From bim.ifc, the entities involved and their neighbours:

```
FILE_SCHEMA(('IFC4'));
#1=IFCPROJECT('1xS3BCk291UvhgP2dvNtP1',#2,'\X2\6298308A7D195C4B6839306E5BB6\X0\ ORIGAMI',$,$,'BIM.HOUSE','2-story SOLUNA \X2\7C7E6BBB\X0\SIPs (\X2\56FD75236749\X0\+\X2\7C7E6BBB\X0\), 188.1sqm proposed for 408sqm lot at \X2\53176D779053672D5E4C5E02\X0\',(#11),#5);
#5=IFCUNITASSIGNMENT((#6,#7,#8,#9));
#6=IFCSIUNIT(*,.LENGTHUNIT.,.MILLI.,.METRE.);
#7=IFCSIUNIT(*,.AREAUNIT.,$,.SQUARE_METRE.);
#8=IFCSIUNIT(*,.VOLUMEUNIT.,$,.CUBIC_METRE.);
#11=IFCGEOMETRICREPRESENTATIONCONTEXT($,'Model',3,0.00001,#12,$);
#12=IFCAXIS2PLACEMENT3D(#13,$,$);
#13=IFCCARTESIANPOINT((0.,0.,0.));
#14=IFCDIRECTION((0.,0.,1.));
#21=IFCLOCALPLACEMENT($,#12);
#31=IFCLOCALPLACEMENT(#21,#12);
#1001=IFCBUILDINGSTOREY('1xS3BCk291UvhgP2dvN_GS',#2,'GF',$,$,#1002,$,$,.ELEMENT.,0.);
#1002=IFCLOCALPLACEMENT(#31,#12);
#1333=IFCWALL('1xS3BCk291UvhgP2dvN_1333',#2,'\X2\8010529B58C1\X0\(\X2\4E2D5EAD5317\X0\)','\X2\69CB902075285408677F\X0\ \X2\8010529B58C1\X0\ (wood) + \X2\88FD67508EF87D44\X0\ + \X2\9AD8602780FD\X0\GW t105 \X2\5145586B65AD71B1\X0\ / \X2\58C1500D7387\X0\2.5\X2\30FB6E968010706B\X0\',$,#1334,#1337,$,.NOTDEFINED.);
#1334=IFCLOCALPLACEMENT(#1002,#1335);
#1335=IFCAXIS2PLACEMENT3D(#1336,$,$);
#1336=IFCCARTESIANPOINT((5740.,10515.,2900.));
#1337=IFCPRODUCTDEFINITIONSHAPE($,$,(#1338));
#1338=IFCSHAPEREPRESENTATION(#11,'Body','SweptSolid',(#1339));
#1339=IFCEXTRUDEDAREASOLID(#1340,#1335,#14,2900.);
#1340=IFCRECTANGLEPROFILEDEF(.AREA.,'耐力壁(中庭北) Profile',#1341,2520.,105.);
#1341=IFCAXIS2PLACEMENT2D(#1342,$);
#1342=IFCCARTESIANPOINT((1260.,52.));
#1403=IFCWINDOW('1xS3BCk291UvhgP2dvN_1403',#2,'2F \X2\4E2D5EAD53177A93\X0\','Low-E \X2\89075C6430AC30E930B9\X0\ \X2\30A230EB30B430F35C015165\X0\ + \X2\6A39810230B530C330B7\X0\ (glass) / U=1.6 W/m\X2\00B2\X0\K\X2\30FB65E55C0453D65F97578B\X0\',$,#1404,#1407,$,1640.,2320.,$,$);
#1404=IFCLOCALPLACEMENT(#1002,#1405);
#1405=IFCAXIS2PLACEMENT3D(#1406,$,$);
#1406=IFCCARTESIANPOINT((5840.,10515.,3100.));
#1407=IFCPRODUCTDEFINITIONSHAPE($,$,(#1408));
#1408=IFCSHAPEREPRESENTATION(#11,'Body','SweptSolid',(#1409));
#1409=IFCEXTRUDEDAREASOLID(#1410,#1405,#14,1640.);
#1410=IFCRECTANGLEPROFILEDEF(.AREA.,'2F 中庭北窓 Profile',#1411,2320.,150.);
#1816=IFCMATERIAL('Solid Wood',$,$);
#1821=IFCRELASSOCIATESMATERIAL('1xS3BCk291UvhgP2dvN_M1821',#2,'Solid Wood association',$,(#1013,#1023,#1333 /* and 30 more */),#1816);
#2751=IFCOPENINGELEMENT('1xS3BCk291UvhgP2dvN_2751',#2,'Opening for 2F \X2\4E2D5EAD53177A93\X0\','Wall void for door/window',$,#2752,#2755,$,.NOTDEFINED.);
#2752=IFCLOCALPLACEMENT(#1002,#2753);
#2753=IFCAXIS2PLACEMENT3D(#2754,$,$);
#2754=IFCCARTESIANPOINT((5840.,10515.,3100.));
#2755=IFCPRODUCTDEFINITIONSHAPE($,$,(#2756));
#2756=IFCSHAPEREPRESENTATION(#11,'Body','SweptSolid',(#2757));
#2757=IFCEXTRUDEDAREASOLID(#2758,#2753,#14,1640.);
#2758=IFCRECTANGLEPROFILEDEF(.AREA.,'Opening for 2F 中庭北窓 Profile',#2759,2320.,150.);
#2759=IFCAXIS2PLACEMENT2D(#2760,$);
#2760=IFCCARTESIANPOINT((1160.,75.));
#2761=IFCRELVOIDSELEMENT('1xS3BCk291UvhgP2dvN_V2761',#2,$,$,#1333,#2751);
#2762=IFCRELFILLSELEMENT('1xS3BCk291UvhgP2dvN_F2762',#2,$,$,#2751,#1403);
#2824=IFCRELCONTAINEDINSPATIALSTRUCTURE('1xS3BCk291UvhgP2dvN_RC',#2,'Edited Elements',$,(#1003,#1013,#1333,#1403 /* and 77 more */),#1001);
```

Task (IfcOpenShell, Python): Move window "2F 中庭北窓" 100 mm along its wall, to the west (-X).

```python
import ifcopenshell
import ifcopenshell.api.geometry
import ifcopenshell.util.placement
import ifcopenshell.util.unit

model = ifcopenshell.open("bim.ifc")
unit_scale = ifcopenshell.util.unit.calculate_unit_scale(model)

window = model.by_guid("1xS3BCk291UvhgP2dvN_1403")
opening = window.FillsVoids[0].RelatingOpeningElement
wall = opening.VoidsElements[0].RelatingBuildingElement

wall_matrix = ifcopenshell.util.placement.get_local_placement(wall.ObjectPlacement)
shift = wall_matrix[:3, 0] * -0.1 / unit_scale
before = ifcopenshell.util.placement.get_local_placement(window.ObjectPlacement)[:3, 3].copy()

# The window is not placed relative to its opening, so move both.
for product in (opening, window):
    matrix = ifcopenshell.util.placement.get_local_placement(product.ObjectPlacement)
    matrix[:3, 3] += shift
    ifcopenshell.api.geometry.edit_object_placement(model, product=product, matrix=matrix, is_si=False)

after = ifcopenshell.util.placement.get_local_placement(window.ObjectPlacement)[:3, 3]
print("window moved by", (after - before).round(3) + 0.0)

model.write("bim_v2.ifc")
```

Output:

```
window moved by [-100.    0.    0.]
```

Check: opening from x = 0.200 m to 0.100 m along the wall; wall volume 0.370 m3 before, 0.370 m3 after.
